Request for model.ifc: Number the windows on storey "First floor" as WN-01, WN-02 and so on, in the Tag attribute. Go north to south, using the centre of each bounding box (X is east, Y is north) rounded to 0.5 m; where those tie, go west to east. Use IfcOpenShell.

First a look at what the model holds.

```python
import ifcopenshell
import ifcopenshell.util.element
import ifcopenshell.util.placement

model = ifcopenshell.open("model.ifc")
print(model.schema)
storey = next(s for s in model.by_type("IfcBuildingStorey") if s.Name == "First floor")
windows = [e for e in ifcopenshell.util.element.get_decomposition(storey) if e.is_a("IfcWindow")]
for e in sorted(windows, key=lambda e: e.id()):
    origin = ifcopenshell.util.placement.get_local_placement(e.ObjectPlacement)[:3, 3]
    print(e.id(), e.Tag, e.Name, origin.round(2) + 0.0, sep=" | ")
```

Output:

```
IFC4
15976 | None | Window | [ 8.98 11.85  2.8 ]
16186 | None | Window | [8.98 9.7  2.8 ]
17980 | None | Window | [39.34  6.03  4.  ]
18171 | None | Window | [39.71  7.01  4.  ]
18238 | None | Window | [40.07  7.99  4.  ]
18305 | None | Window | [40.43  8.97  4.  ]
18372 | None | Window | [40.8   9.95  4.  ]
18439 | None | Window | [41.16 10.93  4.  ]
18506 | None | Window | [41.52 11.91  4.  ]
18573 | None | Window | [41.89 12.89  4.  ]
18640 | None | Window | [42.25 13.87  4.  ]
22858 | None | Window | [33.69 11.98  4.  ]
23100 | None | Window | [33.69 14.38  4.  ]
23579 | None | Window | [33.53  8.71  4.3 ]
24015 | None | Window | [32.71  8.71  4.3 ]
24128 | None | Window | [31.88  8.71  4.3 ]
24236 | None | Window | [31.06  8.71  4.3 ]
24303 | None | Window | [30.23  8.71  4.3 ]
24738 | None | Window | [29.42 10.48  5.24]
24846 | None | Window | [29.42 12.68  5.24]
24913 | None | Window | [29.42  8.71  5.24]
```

```python
import ifcopenshell
import ifcopenshell.geom
import ifcopenshell.util.element
import ifcopenshell.util.shape

model = ifcopenshell.open("model.ifc")
settings = ifcopenshell.geom.settings()
settings.set("use-world-coords", True)


def centre(element):
    shape = ifcopenshell.geom.create_shape(settings, element)
    return ifcopenshell.util.shape.get_bbox_centroid(shape.geometry)


storey = next(s for s in model.by_type("IfcBuildingStorey") if s.Name == "First floor")
windows = [e for e in ifcopenshell.util.element.get_decomposition(storey) if e.is_a("IfcWindow")]

# Insertion points can sit at a corner or the storey origin, so sort by the geometry (in metres).
centres = {e: centre(e) for e in windows}
windows.sort(key=lambda e: (-round(centres[e][1] / 0.5), centres[e][0]))

for i, e in enumerate(windows, start=1):
    number = f"WN-{i:02d}"
    e.Tag = number
    print(e.id(), number)

model.write("model_edited.ifc")
```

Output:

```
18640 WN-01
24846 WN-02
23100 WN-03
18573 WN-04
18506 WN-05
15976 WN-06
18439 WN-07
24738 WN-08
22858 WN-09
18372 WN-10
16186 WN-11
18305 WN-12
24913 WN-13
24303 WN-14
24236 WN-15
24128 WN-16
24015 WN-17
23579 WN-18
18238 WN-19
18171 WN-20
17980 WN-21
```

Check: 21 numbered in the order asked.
